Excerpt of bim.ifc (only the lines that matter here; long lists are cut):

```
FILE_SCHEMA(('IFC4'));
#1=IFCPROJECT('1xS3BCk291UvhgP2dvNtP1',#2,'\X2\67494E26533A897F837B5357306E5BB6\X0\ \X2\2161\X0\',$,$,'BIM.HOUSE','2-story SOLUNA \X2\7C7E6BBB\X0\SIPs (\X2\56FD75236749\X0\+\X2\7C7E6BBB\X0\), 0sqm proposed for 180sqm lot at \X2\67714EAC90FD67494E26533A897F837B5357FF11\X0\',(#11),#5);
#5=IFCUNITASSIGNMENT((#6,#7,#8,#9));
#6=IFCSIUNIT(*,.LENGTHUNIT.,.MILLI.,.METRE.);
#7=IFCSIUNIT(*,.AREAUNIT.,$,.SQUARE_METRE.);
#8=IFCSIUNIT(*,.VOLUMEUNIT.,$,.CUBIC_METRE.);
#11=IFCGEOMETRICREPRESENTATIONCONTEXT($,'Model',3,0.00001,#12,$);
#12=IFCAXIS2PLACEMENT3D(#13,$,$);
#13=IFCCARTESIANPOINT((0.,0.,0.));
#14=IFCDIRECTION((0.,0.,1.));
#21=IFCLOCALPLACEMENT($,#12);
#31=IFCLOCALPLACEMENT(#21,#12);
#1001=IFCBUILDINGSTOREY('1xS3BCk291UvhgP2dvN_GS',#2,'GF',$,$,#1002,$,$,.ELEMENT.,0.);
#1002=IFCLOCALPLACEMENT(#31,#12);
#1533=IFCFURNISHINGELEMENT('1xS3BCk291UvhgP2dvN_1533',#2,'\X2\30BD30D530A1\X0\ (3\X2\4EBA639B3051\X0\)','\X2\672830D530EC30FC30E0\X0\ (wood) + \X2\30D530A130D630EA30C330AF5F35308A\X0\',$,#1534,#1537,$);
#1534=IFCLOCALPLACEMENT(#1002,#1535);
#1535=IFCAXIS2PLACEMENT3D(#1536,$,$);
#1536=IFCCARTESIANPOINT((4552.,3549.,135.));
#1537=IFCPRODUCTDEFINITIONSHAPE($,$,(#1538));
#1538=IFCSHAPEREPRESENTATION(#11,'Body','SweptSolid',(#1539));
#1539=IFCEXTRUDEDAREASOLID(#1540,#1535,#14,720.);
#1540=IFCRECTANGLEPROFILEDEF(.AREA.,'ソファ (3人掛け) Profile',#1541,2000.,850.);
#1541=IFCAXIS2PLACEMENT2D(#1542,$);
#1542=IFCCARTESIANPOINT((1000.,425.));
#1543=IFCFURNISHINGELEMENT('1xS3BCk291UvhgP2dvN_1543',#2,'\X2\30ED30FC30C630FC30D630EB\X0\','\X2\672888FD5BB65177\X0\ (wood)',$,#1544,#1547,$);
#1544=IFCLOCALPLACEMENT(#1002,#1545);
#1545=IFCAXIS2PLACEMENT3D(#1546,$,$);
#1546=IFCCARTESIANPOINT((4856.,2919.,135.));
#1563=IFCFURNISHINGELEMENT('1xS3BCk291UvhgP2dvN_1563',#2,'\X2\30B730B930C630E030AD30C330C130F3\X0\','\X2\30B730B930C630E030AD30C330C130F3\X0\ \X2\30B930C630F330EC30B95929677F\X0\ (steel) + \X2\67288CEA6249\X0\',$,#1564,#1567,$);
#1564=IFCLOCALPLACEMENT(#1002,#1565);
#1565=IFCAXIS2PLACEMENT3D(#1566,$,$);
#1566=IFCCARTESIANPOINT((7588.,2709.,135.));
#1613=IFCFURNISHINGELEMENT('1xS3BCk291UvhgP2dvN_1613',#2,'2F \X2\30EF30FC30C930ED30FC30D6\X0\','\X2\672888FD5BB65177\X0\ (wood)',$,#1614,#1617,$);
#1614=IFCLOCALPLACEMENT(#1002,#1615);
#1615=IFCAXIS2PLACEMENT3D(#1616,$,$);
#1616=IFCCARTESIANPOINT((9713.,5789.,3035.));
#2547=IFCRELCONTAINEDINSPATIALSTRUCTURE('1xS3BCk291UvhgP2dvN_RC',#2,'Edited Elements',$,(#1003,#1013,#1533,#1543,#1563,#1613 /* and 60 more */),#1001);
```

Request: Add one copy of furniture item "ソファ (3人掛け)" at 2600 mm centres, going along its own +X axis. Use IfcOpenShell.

```python
import ifcopenshell
import ifcopenshell.api.geometry
import ifcopenshell.api.root
import ifcopenshell.util.element
import ifcopenshell.util.placement

model = ifcopenshell.open("bim.ifc")


def reuse_history(source, copy):
    """copy_class also copies each property set's owner history, people and application; keep the originals."""
    for rel in copy.IsDefinedBy:
        if rel.is_a("IfcRelDefinesByProperties") and (history := rel.RelatingPropertyDefinition.OwnerHistory):
            rel.RelatingPropertyDefinition.OwnerHistory = source.OwnerHistory
            ifcopenshell.util.element.remove_deep2(model, history)


source = model.by_guid("1xS3BCk291UvhgP2dvN_1533")
base = ifcopenshell.util.placement.get_local_placement(source.ObjectPlacement)
step = base[:3, 0] * 2600.0

for i in range(1, 2):
    copy = ifcopenshell.api.root.copy_class(model, product=source)
    copy.Representation = ifcopenshell.util.element.copy_deep(
        model, source.Representation, exclude=["IfcGeometricRepresentationContext", "IfcRepresentationMap"]
    )
    reuse_history(source, copy)
    matrix = base.copy()
    matrix[:3, 3] += i * step
    print("added at", matrix[:3, 3].round(3) + 0.0)
    ifcopenshell.api.geometry.edit_object_placement(model, product=copy, matrix=matrix, is_si=False)

model.write("bim_updated.ifc")
```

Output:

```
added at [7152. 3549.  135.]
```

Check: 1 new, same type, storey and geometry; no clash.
